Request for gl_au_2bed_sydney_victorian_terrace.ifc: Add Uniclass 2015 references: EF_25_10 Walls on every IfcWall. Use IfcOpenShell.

First a look at what the model holds.

```python
import ifcopenshell

model = ifcopenshell.open("gl_au_2bed_sydney_victorian_terrace.ifc")
print(model.schema)
print("classifications:", [c.Name for c in model.by_type("IfcClassification")])
for ifc_class in ("IfcDoor", "IfcRoof", "IfcStair", "IfcWall", "IfcWindow"):
    print(ifc_class, len(model.by_type(ifc_class)))
```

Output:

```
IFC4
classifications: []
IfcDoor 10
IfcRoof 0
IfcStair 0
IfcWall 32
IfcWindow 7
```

```python
import ifcopenshell
import ifcopenshell.api.classification

model = ifcopenshell.open("gl_au_2bed_sydney_victorian_terrace.ifc")

system = ifcopenshell.api.classification.add_classification(model, classification="Uniclass 2015")

codes = {
    "IfcWall": ("EF_25_10", "Walls"),
}
for ifc_class, (code, name) in codes.items():
    products = model.by_type(ifc_class)
    ifcopenshell.api.classification.add_reference(
        model, products=products, classification=system, identification=code, name=name
    )
    print(code, len(products))

model.write("gl_au_2bed_sydney_victorian_terrace_rev.ifc")
```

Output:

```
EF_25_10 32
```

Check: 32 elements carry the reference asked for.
